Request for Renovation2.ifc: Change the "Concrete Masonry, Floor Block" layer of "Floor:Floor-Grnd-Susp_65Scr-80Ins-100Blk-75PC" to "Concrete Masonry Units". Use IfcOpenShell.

First a look at what the model holds.

```python
import ifcopenshell
import ifcopenshell.util.element

model = ifcopenshell.open("Renovation2.ifc")
print(model.schema)
for layer_set in model.by_type("IfcMaterialLayerSet"):
    if layer_set.LayerSetName == "Floor:Floor-Grnd-Susp_65Scr-80Ins-100Blk-75PC":
        for layer in layer_set.MaterialLayers:
            print(layer.id(), layer.Material and layer.Material.Name, layer.LayerThickness, sep=" | ")
        print(len(ifcopenshell.util.element.get_elements_by_material(model, layer_set)), "elements and types use it")
print(sorted(m.Name for m in model.by_type("IfcMaterial") if m.Name)[:60])
```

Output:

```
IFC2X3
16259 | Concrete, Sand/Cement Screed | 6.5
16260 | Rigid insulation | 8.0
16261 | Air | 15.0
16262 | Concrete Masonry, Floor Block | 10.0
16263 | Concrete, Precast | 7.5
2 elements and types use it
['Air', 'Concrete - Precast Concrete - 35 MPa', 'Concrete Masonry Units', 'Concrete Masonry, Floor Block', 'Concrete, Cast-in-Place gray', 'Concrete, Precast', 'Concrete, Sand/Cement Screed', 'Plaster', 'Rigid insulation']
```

```python
import ifcopenshell
import ifcopenshell.api.material

model = ifcopenshell.open("Renovation2.ifc")

layer_set = next(s for s in model.by_type("IfcMaterialLayerSet") if s.LayerSetName == "Floor:Floor-Grnd-Susp_65Scr-80Ins-100Blk-75PC")
layer = next(l for l in layer_set.MaterialLayers if l.Material and l.Material.Name == "Concrete Masonry, Floor Block")
material = next(m for m in model.by_type("IfcMaterial") if m.Name == "Concrete Masonry Units")

# Point this one layer at the other material; renaming the old one would change it everywhere.
ifcopenshell.api.material.edit_layer(model, layer=layer, attributes={}, material=material)

print([l.Material.Name if l.Material else None for l in layer_set.MaterialLayers])

model.write("Renovation2_v2.ifc")
```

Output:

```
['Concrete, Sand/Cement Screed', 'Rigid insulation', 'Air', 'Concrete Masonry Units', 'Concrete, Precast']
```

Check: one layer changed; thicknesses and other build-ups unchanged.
